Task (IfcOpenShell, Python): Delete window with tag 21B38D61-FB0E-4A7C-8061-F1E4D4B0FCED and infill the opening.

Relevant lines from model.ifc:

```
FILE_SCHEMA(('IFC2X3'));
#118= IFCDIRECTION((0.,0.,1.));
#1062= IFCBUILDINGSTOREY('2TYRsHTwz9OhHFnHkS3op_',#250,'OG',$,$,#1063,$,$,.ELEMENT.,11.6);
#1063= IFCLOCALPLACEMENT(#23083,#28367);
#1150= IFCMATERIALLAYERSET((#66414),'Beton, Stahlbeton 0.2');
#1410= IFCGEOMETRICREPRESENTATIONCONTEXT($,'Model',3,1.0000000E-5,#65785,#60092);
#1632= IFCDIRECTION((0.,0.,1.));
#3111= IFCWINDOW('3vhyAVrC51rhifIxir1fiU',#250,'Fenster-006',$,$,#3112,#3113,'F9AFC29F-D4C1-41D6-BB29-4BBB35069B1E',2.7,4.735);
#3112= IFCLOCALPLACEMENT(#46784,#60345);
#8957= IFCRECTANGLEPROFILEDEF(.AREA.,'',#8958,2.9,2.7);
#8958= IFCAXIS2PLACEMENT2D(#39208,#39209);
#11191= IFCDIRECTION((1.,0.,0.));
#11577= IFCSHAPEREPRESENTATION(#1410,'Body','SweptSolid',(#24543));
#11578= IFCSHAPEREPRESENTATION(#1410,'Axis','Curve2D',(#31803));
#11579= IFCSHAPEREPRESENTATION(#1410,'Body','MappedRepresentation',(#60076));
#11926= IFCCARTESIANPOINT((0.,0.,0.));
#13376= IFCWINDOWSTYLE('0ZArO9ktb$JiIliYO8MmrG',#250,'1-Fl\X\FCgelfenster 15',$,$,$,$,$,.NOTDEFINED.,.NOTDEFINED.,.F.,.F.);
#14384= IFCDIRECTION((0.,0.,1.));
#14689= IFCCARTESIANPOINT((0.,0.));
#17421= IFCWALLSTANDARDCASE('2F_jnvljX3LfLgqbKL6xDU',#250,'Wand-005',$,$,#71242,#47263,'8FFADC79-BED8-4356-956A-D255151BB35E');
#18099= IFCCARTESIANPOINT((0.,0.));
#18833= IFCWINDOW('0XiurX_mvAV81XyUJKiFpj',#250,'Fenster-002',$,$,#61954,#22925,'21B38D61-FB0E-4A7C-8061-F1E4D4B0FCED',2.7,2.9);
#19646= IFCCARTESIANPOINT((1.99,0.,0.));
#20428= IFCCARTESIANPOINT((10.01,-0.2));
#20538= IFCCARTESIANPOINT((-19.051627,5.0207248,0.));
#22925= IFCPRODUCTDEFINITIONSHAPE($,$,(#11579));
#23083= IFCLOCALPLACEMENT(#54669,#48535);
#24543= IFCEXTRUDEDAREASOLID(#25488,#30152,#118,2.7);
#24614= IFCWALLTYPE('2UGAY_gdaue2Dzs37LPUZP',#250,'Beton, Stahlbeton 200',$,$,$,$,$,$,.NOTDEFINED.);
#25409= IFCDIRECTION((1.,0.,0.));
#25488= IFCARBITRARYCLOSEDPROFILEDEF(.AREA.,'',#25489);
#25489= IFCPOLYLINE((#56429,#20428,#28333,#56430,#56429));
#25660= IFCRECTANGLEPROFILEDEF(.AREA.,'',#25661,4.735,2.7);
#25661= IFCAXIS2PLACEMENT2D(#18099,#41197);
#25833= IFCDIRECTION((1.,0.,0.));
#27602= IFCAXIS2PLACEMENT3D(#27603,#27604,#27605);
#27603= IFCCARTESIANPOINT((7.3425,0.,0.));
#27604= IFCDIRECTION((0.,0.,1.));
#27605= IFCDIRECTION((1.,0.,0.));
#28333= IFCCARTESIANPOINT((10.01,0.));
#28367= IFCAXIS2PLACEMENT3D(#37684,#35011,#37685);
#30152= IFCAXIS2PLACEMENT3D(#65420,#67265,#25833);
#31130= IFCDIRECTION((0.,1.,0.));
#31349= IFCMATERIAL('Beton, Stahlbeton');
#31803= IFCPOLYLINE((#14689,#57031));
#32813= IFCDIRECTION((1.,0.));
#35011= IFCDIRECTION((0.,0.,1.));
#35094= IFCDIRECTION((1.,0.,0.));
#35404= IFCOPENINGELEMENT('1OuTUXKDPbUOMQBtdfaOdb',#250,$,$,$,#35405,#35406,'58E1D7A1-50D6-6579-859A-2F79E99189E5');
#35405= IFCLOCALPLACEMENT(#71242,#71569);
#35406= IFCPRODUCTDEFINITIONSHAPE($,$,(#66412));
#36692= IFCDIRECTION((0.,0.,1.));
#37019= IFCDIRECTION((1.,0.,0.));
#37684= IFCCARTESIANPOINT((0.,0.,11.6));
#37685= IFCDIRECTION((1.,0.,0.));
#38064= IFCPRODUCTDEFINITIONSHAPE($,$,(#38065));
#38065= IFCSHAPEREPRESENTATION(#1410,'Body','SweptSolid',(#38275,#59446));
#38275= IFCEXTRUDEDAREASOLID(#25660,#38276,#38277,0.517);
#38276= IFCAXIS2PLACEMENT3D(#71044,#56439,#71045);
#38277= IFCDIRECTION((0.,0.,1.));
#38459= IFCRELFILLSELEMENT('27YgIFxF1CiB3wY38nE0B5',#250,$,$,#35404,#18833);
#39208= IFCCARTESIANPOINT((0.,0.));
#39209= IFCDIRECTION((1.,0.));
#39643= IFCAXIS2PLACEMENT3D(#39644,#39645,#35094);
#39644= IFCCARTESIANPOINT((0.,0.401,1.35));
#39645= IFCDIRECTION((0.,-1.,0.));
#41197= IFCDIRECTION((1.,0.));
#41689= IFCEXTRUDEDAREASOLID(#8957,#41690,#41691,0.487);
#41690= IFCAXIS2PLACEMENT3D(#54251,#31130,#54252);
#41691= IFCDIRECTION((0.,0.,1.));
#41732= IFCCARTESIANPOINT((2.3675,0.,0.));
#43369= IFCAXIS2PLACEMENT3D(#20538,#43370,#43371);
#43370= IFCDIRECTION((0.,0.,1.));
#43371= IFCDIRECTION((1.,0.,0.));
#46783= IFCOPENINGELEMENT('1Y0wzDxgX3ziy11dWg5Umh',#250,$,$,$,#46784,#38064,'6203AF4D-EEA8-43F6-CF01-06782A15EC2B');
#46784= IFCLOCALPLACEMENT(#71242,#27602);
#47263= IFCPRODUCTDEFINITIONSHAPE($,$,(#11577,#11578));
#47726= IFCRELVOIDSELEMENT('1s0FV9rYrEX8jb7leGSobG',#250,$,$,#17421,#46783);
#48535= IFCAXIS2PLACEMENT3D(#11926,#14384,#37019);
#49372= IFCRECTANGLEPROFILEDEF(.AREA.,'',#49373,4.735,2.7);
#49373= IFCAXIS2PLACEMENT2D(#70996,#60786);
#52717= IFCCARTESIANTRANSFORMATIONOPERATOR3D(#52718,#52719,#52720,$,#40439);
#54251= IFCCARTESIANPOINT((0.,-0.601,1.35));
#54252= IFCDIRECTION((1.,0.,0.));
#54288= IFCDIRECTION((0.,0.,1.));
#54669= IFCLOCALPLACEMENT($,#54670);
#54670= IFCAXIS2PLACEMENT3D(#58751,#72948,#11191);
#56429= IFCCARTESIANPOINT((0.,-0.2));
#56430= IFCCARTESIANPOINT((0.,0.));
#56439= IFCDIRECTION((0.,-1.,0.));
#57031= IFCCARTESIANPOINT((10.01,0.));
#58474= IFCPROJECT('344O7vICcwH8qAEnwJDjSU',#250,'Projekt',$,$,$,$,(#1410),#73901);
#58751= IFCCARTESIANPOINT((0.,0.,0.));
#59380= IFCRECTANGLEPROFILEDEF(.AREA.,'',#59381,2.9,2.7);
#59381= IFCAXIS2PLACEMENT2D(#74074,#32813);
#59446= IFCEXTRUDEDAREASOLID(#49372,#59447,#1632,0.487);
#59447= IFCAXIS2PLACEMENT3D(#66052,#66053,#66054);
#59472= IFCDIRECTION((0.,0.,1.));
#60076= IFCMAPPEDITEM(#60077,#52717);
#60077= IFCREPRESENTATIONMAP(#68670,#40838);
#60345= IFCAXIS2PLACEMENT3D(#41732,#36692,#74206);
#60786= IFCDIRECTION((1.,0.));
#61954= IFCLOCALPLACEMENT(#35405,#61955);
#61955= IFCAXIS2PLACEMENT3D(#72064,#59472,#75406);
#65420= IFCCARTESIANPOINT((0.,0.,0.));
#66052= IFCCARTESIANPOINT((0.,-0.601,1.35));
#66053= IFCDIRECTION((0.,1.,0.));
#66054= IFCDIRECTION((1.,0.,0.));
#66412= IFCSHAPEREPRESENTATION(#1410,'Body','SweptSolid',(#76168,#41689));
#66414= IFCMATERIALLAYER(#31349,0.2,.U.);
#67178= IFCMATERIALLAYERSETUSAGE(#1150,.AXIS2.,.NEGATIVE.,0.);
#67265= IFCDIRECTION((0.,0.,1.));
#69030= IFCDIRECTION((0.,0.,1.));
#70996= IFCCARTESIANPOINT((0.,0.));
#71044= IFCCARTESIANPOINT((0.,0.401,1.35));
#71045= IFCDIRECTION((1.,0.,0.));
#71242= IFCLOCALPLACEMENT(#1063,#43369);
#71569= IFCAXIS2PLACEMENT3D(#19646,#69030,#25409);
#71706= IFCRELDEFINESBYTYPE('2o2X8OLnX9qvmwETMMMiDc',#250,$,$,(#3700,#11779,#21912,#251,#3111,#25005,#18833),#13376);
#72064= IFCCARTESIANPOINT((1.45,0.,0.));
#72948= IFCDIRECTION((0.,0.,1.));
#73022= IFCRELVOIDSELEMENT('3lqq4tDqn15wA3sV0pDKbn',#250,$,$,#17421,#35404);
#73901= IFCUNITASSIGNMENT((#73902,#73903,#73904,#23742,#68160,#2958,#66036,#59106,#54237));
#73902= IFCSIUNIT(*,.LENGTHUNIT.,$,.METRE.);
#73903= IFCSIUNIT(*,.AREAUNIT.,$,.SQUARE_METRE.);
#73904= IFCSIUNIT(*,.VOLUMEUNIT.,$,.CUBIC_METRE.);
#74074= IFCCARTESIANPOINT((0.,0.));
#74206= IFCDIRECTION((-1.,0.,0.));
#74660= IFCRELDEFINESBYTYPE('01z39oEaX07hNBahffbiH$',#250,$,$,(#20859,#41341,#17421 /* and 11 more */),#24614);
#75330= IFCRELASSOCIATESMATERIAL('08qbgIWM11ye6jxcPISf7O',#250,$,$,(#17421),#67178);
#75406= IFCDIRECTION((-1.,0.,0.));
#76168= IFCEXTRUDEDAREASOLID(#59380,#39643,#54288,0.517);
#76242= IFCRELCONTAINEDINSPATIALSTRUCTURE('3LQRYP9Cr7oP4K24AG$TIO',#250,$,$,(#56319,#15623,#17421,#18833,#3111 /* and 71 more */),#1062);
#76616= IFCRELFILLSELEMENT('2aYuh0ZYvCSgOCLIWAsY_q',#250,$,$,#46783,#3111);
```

```python
import ifcopenshell
import ifcopenshell.api.feature
import ifcopenshell.api.root
import ifcopenshell.geom
import ifcopenshell.util.shape

model = ifcopenshell.open("model.ifc")
settings = ifcopenshell.geom.settings()


def volume(element):
    """Net volume in cubic metres, openings subtracted."""
    shape = ifcopenshell.geom.create_shape(settings, element)
    return ifcopenshell.util.shape.get_volume(shape.geometry)


window = model.by_guid("0XiurX_mvAV81XyUJKiFpj")
opening = window.FillsVoids[0].RelatingOpeningElement
wall = opening.VoidsElements[0].RelatingBuildingElement
before = volume(wall)

ifcopenshell.api.root.remove_product(model, product=window)
ifcopenshell.api.feature.remove_feature(model, feature=opening)

after = volume(wall)

print(f"wall volume {before:.3f} -> {after:.3f} m3")

model.write("model_v2.ifc")
```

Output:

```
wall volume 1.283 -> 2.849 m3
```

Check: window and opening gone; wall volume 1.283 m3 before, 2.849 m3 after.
